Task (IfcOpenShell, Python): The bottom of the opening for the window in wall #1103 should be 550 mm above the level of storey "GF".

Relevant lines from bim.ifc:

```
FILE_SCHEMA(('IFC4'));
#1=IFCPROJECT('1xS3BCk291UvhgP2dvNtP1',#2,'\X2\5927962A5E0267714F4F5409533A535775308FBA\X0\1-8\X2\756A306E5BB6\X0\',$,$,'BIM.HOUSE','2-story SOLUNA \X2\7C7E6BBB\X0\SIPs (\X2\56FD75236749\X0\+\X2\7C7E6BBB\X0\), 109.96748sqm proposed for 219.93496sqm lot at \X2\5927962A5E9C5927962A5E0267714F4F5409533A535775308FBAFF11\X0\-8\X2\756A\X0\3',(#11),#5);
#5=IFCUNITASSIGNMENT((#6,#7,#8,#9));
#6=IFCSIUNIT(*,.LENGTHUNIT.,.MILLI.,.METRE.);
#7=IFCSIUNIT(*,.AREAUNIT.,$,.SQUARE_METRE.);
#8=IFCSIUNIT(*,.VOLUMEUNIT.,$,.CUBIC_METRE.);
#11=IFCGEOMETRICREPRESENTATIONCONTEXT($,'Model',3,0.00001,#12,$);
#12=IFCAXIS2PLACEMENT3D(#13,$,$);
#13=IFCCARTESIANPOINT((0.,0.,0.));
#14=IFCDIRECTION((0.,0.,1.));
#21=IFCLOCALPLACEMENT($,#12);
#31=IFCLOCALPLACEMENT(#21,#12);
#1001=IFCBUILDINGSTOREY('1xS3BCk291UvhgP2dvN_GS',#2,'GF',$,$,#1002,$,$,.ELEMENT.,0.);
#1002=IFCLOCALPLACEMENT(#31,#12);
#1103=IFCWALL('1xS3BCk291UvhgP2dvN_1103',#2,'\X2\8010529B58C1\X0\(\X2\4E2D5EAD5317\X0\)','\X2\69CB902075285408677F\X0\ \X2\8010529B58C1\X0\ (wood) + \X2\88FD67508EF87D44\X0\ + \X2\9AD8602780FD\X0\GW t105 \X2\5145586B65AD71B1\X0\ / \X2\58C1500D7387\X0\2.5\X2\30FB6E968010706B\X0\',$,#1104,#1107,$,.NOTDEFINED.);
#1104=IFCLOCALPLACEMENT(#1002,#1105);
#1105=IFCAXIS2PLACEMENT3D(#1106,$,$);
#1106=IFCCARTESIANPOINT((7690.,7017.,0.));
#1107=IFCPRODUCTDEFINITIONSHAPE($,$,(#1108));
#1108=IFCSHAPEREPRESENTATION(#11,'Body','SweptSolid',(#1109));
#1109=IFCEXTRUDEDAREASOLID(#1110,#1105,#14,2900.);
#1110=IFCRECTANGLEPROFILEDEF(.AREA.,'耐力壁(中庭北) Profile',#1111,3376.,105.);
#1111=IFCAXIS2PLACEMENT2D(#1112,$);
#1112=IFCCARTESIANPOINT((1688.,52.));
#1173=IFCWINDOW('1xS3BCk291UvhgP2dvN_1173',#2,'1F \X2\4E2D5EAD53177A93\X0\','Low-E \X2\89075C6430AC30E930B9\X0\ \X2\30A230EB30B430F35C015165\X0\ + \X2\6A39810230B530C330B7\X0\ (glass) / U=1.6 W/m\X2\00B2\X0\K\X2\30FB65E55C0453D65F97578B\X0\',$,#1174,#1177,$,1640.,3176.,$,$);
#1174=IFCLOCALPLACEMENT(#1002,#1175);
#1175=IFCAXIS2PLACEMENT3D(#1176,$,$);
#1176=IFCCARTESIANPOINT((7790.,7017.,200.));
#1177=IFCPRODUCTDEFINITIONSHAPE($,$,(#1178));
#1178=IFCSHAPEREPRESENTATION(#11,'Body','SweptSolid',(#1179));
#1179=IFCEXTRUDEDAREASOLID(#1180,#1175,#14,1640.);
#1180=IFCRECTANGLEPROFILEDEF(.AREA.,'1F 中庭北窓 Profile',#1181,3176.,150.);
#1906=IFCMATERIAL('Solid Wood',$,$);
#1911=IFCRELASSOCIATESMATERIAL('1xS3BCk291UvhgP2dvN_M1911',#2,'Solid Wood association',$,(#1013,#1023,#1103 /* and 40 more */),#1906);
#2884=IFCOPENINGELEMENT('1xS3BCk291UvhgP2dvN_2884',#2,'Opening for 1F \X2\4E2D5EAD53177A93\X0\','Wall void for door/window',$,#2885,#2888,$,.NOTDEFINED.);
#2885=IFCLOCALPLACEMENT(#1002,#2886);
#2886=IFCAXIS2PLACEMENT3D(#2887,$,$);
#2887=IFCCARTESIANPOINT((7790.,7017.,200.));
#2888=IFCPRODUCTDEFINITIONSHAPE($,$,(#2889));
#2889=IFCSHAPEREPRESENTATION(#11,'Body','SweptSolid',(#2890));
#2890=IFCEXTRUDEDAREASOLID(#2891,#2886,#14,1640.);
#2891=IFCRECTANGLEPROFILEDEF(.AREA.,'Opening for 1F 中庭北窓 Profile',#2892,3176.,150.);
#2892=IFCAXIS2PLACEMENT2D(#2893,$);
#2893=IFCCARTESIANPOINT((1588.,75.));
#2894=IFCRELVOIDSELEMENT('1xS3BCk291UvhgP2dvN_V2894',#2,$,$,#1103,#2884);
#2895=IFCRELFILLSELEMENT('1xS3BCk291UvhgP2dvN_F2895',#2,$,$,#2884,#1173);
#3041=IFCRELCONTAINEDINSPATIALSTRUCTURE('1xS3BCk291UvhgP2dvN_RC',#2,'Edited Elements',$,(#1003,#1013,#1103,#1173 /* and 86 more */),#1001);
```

```python
import numpy as np
import ifcopenshell
import ifcopenshell.api.geometry
import ifcopenshell.geom
import ifcopenshell.util.element
import ifcopenshell.util.placement
import ifcopenshell.util.shape
import ifcopenshell.util.unit

model = ifcopenshell.open("bim.ifc")
unit_scale = ifcopenshell.util.unit.calculate_unit_scale(model)

window = model.by_id(1173)
opening = window.FillsVoids[0].RelatingOpeningElement
storey = ifcopenshell.util.element.get_container(window, ifc_class="IfcBuildingStorey")
level = ifcopenshell.util.placement.get_local_placement(storey.ObjectPlacement)[2, 3]

# The opening's origin need not be at the sill, so measure its lowest point.
shape = ifcopenshell.geom.create_shape(ifcopenshell.geom.settings(), opening)
bottom = ifcopenshell.util.shape.get_shape_bottom_elevation(shape, shape.geometry) / unit_scale
dz = level + 0.55 / unit_scale - bottom

shift = np.array([0.0, 0.0, dz])
# The window is not placed relative to its opening, so move both.
for product in (opening, window):
    matrix = ifcopenshell.util.placement.get_local_placement(product.ObjectPlacement)
    matrix[:3, 3] += shift
    ifcopenshell.api.geometry.edit_object_placement(model, product=product, matrix=matrix, is_si=False)

print(f"moved by {dz * unit_scale:+.3f} m")

model.write("bim_updated.ifc")
```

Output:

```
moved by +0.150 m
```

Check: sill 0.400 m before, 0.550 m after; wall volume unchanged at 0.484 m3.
